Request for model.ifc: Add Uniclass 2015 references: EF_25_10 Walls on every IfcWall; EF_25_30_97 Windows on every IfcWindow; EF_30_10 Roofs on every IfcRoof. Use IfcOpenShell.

First a look at what the model holds.

```python
import ifcopenshell

model = ifcopenshell.open("model.ifc")
print(model.schema)
print("classifications:", [c.Name for c in model.by_type("IfcClassification")])
for ifc_class in ("IfcDoor", "IfcRoof", "IfcStair", "IfcWall", "IfcWindow"):
    print(ifc_class, len(model.by_type(ifc_class)))
```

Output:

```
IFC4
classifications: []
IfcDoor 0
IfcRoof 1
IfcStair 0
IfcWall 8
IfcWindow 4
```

```python
import ifcopenshell
import ifcopenshell.api.classification

model = ifcopenshell.open("model.ifc")

system = ifcopenshell.api.classification.add_classification(model, classification="Uniclass 2015")

codes = {
    "IfcWall": ("EF_25_10", "Walls"),
    "IfcWindow": ("EF_25_30_97", "Windows"),
    "IfcRoof": ("EF_30_10", "Roofs"),
}
for ifc_class, (code, name) in codes.items():
    products = model.by_type(ifc_class)
    ifcopenshell.api.classification.add_reference(
        model, products=products, classification=system, identification=code, name=name
    )
    print(code, len(products))

model.write("model_rev.ifc")
```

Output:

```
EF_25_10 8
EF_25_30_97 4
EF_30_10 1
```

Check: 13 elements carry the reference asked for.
